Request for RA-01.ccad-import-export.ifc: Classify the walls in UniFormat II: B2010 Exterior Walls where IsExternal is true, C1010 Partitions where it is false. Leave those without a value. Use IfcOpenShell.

First a look at what the model holds.

```python
import ifcopenshell
import ifcopenshell.util.element

model = ifcopenshell.open("RA-01.ccad-import-export.ifc")
print(model.schema)
print("classifications:", [c.Name for c in model.by_type("IfcClassification")])
values = [ifcopenshell.util.element.get_pset(e, "Pset_WallCommon", "IsExternal") for e in model.by_type("IfcWall")]
for value in (True, False, None):
    print("IsExternal", value, values.count(value))
```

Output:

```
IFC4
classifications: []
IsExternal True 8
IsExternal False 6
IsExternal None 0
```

```python
import ifcopenshell
import ifcopenshell.api.classification
import ifcopenshell.util.element

model = ifcopenshell.open("RA-01.ccad-import-export.ifc")

system = ifcopenshell.api.classification.add_classification(model, classification="UniFormat II")

walls = model.by_type("IfcWall")
external = {e: ifcopenshell.util.element.get_pset(e, "Pset_WallCommon", "IsExternal") for e in walls}
for flag, code, name in ((True, "B2010", "Exterior Walls"), (False, "C1010", "Partitions")):
    products = [e for e in walls if external[e] is flag]
    ifcopenshell.api.classification.add_reference(
        model, products=products, classification=system, identification=code, name=name
    )
    print(code, len(products))

model.write("RA-01.ccad-import-export_rev.ifc")
```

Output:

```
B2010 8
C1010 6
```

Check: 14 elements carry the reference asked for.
